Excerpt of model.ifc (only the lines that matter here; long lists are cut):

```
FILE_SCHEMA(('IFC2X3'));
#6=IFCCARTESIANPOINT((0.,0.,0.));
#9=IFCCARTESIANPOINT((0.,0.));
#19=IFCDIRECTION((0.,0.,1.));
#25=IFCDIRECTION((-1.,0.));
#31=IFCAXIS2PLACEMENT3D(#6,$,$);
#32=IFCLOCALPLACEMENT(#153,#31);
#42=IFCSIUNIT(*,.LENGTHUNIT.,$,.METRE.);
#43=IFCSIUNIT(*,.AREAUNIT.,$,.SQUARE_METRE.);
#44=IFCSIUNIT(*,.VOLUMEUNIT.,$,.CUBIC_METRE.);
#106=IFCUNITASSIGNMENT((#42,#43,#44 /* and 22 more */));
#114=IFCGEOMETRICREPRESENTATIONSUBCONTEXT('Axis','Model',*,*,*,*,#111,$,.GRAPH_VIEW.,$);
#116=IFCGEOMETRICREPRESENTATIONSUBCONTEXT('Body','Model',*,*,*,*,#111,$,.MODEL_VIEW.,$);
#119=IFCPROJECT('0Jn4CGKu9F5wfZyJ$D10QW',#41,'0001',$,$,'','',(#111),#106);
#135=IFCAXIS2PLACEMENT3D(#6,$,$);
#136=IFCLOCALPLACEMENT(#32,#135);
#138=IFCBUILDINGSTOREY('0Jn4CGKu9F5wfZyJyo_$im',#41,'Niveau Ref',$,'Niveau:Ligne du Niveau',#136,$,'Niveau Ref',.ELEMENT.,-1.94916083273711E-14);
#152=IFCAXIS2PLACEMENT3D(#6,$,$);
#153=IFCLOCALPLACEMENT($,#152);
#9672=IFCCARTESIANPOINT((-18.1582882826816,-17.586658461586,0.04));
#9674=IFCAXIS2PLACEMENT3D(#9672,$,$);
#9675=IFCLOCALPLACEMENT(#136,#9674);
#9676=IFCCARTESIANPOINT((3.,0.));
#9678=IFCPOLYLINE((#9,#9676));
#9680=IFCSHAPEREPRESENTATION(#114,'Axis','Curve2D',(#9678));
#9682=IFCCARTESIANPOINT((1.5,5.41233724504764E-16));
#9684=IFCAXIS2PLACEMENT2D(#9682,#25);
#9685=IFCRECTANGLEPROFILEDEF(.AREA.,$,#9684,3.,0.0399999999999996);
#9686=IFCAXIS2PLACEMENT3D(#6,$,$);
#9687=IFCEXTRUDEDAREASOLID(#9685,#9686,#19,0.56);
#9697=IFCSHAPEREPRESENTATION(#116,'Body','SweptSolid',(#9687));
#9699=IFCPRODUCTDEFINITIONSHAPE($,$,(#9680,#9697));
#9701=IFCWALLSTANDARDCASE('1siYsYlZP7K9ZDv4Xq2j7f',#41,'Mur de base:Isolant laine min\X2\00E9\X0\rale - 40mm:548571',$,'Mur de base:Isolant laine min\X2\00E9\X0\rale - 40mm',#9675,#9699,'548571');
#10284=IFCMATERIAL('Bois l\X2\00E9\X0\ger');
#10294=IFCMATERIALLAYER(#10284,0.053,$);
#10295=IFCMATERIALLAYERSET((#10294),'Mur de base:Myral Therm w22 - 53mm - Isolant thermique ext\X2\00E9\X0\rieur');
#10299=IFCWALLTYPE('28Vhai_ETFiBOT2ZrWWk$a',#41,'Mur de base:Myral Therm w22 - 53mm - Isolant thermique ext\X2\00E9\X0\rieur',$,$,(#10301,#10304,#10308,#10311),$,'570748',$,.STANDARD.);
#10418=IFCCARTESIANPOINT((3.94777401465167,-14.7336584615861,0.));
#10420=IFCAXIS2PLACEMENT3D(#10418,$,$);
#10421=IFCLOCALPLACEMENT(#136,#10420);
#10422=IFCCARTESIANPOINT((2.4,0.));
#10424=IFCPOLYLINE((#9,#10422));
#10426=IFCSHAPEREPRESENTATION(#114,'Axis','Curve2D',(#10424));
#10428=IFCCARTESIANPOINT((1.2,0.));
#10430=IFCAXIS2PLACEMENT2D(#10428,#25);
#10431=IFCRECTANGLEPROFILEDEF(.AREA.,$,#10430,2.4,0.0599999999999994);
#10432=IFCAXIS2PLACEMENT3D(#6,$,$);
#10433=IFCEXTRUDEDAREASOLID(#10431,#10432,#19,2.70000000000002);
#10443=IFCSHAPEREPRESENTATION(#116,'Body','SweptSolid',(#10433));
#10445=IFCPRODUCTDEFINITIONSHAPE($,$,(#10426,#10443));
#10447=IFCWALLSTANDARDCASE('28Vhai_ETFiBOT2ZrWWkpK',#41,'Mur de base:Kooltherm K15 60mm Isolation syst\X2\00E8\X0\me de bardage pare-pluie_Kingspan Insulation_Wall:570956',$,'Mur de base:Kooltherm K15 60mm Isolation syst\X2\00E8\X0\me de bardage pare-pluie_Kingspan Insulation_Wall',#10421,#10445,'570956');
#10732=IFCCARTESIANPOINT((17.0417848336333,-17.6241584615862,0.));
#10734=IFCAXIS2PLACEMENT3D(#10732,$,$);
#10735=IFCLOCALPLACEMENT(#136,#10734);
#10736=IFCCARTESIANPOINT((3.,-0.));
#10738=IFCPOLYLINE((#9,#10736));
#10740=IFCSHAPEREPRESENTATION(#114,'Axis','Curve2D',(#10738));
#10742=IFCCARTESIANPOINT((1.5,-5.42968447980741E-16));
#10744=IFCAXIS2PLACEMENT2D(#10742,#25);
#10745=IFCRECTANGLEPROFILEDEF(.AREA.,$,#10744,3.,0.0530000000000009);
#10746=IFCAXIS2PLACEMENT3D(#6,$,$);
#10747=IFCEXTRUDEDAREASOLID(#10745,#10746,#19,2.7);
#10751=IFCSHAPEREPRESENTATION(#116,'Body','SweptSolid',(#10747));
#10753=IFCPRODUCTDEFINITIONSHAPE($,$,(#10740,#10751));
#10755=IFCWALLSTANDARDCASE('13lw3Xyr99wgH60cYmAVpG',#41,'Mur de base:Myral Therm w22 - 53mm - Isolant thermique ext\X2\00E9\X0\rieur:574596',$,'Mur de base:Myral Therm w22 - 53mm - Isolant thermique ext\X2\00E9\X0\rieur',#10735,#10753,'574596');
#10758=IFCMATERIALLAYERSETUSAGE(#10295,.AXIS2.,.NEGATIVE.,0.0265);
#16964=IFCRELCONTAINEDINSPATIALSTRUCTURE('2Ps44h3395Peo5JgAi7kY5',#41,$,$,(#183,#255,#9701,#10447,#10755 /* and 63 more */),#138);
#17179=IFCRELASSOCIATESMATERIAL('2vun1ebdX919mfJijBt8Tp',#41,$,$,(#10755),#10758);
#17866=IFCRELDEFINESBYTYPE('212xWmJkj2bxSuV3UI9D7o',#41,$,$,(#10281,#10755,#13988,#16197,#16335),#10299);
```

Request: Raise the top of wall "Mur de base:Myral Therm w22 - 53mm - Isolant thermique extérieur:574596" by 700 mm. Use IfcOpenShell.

```python
import ifcopenshell
import ifcopenshell.geom
import ifcopenshell.util.representation
import ifcopenshell.util.shape
import ifcopenshell.util.unit

model = ifcopenshell.open("model.ifc")
unit_scale = ifcopenshell.util.unit.calculate_unit_scale(model)
settings = ifcopenshell.geom.settings()


def volume(element):
    """Net volume in cubic metres, openings subtracted."""
    shape = ifcopenshell.geom.create_shape(settings, element)
    return ifcopenshell.util.shape.get_volume(shape.geometry)


wall = model.by_guid("13lw3Xyr99wgH60cYmAVpG")
before = volume(wall)

body = ifcopenshell.util.representation.get_representation(wall, "Model", "Body")
solid = body.Items[0]
old_height = solid.Depth
solid.Depth += 0.7 / unit_scale
after = volume(wall)

print(f"height {old_height:g} -> {solid.Depth:g}, volume {before:.3f} -> {after:.3f} m3")

model.write("model_updated.ifc")
```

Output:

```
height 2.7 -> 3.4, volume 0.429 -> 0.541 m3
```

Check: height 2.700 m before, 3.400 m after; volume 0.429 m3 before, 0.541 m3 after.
